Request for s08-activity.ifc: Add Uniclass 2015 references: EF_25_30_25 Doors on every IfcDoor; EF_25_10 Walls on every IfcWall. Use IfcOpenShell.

First a look at what the model holds.

```python
import ifcopenshell

model = ifcopenshell.open("s08-activity.ifc")
print(model.schema)
print("classifications:", [c.Name for c in model.by_type("IfcClassification")])
for ifc_class in ("IfcDoor", "IfcRoof", "IfcStair", "IfcWall", "IfcWindow"):
    print(ifc_class, len(model.by_type(ifc_class)))
```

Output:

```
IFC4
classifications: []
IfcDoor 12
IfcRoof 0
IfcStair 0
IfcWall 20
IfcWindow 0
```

```python
import ifcopenshell
import ifcopenshell.api.classification

model = ifcopenshell.open("s08-activity.ifc")

system = ifcopenshell.api.classification.add_classification(model, classification="Uniclass 2015")

codes = {
    "IfcDoor": ("EF_25_30_25", "Doors"),
    "IfcWall": ("EF_25_10", "Walls"),
}
for ifc_class, (code, name) in codes.items():
    products = model.by_type(ifc_class)
    ifcopenshell.api.classification.add_reference(
        model, products=products, classification=system, identification=code, name=name
    )
    print(code, len(products))

model.write("s08-activity_v2.ifc")
```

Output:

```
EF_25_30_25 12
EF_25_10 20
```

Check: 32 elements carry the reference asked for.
